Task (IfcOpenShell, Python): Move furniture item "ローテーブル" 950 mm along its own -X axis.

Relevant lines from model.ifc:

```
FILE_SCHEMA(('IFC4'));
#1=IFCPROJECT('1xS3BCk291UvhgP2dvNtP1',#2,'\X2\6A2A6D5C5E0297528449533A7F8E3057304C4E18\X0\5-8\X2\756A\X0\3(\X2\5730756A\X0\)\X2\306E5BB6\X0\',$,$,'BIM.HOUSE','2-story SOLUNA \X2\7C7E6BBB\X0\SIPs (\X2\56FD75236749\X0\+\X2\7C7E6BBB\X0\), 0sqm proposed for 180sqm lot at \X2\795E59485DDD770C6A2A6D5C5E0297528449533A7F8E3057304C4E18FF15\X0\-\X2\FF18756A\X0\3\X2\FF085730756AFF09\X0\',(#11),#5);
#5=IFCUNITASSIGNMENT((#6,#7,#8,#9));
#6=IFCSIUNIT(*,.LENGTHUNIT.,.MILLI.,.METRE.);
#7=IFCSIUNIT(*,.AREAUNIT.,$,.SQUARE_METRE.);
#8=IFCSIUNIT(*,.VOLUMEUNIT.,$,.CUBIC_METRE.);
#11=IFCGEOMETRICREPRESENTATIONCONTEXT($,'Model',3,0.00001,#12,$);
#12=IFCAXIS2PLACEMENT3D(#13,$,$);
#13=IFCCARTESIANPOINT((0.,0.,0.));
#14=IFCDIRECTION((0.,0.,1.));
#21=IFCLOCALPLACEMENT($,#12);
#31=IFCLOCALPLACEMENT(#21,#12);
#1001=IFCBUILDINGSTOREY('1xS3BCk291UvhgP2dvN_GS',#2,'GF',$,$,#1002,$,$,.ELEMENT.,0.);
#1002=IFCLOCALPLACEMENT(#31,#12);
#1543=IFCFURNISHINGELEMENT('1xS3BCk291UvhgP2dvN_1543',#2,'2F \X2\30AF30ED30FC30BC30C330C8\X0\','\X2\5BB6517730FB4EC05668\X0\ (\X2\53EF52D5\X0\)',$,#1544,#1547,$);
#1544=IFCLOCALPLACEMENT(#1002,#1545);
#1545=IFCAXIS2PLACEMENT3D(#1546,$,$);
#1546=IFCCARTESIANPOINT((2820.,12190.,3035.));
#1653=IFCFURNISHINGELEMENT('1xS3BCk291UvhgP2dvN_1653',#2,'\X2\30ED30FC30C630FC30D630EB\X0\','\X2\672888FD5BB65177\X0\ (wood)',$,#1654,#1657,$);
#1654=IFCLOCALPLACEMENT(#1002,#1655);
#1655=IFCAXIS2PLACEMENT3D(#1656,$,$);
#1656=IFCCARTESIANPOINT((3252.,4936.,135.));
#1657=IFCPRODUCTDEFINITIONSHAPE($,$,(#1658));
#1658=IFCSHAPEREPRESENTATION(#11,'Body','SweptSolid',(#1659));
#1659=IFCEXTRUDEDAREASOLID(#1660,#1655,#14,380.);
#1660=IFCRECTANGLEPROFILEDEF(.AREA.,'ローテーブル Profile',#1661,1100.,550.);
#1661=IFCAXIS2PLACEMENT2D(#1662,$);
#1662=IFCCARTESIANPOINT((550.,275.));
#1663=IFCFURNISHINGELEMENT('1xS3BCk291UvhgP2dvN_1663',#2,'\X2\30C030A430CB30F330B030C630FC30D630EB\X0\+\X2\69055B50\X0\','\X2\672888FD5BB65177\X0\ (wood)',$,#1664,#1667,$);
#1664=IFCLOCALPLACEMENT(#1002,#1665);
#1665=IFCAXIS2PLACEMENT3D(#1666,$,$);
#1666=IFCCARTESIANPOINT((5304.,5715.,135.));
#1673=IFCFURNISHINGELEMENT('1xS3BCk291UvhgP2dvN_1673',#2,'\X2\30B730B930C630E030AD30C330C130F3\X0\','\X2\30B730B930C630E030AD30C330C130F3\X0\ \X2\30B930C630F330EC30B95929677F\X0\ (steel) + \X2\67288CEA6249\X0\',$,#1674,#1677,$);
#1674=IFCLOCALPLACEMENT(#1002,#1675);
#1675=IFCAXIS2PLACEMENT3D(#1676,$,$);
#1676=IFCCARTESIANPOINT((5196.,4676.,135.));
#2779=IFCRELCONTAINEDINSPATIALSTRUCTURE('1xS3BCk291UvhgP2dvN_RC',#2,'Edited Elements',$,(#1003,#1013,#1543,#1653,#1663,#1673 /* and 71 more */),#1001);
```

```python
import ifcopenshell
import ifcopenshell.api.geometry
import ifcopenshell.util.placement
import ifcopenshell.util.unit

model = ifcopenshell.open("model.ifc")
unit_scale = ifcopenshell.util.unit.calculate_unit_scale(model)

item = model.by_guid("1xS3BCk291UvhgP2dvN_1653")
matrix = ifcopenshell.util.placement.get_local_placement(item.ObjectPlacement)
matrix[:3, 3] -= matrix[:3, 0] * 0.95 / unit_scale
ifcopenshell.api.geometry.edit_object_placement(model, product=item, matrix=matrix, is_si=False)

print(ifcopenshell.util.placement.get_local_placement(item.ObjectPlacement).round(3) + 0.0)

model.write("model_updated.ifc")
```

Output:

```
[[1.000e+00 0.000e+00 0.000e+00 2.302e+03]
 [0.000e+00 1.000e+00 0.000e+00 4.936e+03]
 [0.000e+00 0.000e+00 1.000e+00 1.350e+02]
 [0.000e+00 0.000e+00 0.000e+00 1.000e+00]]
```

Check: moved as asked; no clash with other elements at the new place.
